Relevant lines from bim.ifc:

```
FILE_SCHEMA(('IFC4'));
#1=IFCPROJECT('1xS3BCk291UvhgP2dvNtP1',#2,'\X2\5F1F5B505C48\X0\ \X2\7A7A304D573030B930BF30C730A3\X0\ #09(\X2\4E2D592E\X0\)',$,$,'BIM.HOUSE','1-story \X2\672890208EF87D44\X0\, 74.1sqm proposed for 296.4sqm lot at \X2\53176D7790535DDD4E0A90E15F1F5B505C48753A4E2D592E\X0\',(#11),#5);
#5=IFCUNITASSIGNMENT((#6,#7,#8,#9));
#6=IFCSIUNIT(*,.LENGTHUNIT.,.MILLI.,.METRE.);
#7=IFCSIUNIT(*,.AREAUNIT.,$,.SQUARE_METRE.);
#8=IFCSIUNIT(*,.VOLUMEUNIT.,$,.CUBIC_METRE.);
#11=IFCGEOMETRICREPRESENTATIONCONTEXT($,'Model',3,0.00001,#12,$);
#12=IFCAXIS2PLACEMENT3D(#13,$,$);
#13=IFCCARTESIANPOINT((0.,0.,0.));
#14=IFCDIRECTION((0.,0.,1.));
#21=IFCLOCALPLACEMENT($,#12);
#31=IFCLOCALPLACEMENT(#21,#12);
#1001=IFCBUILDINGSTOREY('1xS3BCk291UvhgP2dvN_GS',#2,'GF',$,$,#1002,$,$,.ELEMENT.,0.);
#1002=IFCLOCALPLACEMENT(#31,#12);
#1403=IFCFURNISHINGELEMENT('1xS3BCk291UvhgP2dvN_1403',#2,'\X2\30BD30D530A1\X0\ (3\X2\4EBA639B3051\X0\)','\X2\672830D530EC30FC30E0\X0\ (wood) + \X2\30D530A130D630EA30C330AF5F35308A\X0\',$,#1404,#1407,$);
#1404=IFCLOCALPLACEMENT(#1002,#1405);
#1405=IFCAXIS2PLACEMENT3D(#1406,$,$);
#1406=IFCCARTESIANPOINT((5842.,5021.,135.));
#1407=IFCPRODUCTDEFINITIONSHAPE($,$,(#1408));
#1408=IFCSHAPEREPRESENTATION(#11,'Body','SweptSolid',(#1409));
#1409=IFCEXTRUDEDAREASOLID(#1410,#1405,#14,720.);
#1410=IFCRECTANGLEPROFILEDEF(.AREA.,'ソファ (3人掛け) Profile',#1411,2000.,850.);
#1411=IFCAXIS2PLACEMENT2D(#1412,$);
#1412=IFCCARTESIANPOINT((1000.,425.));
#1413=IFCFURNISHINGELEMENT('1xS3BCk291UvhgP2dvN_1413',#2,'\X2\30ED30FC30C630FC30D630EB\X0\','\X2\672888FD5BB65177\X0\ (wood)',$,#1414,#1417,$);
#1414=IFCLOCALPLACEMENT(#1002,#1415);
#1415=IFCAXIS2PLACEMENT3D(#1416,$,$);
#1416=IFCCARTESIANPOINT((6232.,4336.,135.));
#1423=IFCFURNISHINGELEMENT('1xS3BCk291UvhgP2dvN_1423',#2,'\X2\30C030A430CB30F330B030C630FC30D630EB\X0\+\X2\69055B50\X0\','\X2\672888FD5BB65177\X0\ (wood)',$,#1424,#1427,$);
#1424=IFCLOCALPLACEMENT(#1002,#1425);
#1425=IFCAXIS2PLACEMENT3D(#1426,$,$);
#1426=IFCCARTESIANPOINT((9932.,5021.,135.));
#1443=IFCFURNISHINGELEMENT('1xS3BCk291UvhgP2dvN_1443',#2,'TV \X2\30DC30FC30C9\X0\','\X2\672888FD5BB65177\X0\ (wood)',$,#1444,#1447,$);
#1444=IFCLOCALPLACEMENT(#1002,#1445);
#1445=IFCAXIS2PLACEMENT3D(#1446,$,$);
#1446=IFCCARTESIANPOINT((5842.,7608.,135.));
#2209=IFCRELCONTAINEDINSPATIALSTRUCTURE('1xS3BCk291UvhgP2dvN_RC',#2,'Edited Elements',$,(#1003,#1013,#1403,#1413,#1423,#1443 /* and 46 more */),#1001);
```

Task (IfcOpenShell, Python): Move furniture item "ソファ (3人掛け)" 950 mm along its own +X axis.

```python
import ifcopenshell
import ifcopenshell.api.geometry
import ifcopenshell.util.placement

model = ifcopenshell.open("bim.ifc")

item = model.by_id(1403)
matrix = ifcopenshell.util.placement.get_local_placement(item.ObjectPlacement)
matrix[:3, 3] += matrix[:3, 0] * 950.0
ifcopenshell.api.geometry.edit_object_placement(model, product=item, matrix=matrix, is_si=False)

print(ifcopenshell.util.placement.get_local_placement(item.ObjectPlacement).round(3) + 0.0)

model.write("bim_rev.ifc")
```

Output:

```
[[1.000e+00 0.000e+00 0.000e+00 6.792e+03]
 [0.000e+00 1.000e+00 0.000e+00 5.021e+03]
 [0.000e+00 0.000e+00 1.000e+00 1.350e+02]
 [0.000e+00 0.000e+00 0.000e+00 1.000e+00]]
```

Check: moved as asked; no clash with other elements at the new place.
